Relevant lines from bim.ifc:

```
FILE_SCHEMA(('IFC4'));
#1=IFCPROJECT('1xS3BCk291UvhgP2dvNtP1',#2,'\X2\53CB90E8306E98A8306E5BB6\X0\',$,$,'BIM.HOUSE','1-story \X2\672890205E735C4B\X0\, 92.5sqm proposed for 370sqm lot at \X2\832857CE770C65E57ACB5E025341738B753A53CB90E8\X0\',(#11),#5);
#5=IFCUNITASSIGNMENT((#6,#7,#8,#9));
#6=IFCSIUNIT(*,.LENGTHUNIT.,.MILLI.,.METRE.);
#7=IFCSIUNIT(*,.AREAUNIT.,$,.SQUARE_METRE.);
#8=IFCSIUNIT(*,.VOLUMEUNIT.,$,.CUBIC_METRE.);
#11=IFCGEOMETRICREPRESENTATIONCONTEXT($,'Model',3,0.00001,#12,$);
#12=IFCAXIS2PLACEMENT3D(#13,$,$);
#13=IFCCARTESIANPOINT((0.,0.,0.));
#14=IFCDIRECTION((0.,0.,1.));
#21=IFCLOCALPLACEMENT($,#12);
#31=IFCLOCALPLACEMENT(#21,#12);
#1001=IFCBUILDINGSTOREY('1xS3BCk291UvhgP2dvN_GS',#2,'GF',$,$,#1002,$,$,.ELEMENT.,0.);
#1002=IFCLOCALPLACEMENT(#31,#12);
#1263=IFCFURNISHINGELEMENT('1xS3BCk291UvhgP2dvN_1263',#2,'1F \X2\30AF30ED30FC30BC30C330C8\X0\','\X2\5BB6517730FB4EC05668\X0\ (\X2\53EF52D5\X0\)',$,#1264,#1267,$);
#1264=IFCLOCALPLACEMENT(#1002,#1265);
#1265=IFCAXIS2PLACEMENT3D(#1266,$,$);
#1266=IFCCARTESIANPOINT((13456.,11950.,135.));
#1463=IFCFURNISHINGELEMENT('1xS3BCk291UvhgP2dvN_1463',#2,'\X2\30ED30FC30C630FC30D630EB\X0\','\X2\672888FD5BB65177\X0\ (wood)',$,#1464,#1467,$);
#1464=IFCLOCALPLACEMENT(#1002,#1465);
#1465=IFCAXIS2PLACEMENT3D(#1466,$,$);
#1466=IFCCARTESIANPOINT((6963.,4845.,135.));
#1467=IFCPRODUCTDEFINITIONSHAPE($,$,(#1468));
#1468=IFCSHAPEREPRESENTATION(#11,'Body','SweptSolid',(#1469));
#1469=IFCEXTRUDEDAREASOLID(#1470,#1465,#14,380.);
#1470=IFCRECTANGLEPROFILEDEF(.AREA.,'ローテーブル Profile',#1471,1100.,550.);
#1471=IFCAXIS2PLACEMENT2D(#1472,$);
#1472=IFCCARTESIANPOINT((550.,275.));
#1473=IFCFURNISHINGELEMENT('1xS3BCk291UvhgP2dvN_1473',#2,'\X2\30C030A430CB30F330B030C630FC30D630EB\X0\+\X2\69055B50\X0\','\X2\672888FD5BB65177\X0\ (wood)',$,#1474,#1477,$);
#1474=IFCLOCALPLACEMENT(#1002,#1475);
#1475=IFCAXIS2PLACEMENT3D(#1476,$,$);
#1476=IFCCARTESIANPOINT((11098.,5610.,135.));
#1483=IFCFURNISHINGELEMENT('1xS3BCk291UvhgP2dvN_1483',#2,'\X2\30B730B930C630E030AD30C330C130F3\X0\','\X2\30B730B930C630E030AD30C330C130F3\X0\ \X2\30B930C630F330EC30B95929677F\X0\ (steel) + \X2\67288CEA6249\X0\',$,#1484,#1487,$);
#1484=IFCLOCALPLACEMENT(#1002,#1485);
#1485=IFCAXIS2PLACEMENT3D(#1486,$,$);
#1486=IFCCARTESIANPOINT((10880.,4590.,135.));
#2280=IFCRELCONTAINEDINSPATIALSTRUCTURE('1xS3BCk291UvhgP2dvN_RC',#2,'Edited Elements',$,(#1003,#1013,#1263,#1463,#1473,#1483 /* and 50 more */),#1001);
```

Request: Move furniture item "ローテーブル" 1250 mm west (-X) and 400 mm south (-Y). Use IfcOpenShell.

```python
import ifcopenshell
import ifcopenshell.api.geometry
import ifcopenshell.util.placement

model = ifcopenshell.open("bim.ifc")

item = model.by_guid("1xS3BCk291UvhgP2dvN_1463")
matrix = ifcopenshell.util.placement.get_local_placement(item.ObjectPlacement)
matrix[0, 3] -= 1250.0
matrix[1, 3] -= 400.0
ifcopenshell.api.geometry.edit_object_placement(model, product=item, matrix=matrix, is_si=False)

print(ifcopenshell.util.placement.get_local_placement(item.ObjectPlacement).round(3) + 0.0)

model.write("bim-out.ifc")
```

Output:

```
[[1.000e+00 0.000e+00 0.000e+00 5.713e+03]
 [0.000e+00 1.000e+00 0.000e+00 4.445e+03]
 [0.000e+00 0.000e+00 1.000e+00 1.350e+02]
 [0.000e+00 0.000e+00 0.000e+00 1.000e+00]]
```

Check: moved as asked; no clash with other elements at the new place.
